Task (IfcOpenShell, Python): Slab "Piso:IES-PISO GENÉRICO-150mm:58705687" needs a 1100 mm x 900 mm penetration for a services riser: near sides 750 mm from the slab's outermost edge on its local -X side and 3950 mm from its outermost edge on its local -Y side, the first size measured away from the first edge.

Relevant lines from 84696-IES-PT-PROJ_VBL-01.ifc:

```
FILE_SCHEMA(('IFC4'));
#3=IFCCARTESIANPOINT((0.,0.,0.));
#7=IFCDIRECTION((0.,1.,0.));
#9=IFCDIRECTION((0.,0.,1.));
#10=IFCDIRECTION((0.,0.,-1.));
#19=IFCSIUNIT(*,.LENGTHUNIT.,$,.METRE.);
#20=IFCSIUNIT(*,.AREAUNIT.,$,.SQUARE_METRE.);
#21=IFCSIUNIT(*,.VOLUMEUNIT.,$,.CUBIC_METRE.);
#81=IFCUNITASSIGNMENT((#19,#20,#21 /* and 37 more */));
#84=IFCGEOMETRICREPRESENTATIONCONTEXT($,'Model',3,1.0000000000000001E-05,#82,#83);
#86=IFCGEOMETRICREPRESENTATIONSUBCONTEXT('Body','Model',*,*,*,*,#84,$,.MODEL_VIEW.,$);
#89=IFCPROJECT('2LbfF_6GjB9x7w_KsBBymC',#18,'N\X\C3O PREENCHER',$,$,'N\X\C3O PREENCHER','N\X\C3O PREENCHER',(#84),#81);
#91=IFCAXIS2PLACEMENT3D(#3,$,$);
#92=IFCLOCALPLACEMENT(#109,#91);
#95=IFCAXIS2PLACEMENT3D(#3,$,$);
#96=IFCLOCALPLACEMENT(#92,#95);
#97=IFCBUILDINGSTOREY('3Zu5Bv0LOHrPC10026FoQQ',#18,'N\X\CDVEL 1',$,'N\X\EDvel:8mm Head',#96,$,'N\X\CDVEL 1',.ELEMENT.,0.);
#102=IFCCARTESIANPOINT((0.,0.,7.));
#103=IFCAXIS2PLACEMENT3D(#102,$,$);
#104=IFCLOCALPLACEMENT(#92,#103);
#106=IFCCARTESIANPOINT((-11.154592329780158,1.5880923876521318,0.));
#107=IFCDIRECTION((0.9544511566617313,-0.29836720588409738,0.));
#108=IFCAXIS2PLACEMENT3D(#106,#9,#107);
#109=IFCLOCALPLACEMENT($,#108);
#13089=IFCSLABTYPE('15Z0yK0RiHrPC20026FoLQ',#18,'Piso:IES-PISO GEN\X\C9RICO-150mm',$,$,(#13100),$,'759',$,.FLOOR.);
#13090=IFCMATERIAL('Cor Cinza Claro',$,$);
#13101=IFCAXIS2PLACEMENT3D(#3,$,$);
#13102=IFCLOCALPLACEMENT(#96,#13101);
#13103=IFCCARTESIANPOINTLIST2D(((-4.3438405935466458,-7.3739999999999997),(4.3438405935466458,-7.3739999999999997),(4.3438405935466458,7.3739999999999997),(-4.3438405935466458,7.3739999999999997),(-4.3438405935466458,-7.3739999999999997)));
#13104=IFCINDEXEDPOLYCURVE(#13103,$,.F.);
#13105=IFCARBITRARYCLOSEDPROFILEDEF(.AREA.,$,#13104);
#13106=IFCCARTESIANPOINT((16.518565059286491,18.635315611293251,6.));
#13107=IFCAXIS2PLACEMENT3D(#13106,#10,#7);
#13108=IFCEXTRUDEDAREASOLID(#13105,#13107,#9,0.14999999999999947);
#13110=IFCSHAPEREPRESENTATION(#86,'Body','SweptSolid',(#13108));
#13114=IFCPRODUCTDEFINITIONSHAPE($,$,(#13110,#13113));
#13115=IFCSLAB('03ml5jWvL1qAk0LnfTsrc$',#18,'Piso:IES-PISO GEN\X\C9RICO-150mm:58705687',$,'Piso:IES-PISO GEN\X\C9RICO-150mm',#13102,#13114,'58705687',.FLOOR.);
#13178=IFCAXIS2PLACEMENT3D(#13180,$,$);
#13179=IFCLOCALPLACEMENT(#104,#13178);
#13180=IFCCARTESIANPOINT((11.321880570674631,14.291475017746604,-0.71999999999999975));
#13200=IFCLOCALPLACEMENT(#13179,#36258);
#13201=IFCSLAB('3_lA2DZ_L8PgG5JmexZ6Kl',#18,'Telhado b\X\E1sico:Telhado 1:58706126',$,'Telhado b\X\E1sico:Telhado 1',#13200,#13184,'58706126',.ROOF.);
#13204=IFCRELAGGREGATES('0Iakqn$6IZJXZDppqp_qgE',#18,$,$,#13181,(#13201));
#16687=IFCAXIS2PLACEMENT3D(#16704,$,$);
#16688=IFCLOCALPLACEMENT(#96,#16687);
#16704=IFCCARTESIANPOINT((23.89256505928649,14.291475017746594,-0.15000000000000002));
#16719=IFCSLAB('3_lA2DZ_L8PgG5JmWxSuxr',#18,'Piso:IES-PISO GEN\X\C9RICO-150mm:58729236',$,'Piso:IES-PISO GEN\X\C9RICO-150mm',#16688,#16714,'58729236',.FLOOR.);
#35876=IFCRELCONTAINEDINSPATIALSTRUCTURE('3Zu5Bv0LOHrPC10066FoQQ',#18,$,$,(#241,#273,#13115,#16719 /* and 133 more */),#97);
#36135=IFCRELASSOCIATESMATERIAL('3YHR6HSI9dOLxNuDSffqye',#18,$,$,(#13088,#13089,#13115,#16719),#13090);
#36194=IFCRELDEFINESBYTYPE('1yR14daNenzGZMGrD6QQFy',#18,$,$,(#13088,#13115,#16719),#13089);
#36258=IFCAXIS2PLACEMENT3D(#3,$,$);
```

```python
import numpy as np
import ifcopenshell
import ifcopenshell.api.feature
import ifcopenshell.api.geometry
import ifcopenshell.api.root
import ifcopenshell.geom
import ifcopenshell.util.placement
import ifcopenshell.util.representation
import ifcopenshell.util.shape
import ifcopenshell.util.unit

model = ifcopenshell.open("84696-IES-PT-PROJ_VBL-01.ifc")
unit_scale = ifcopenshell.util.unit.calculate_unit_scale(model)
settings = ifcopenshell.geom.settings()


def volume(element):
    """Net volume in cubic metres, openings subtracted."""
    shape = ifcopenshell.geom.create_shape(settings, element)
    return ifcopenshell.util.shape.get_volume(shape.geometry)


slab = model.by_guid("03ml5jWvL1qAk0LnfTsrc$")
before = volume(slab)

# Extent in the slab's own axes, in metres. The edges named are its -X and -Y sides.
slab_shape = ifcopenshell.geom.create_shape(settings, slab)
vertices = ifcopenshell.util.shape.get_vertices(slab_shape.geometry)
x_min, y_min, bottom = vertices.min(axis=0)
top = vertices[:, 2].max()

opening = ifcopenshell.api.root.create_entity(model, ifc_class="IfcOpeningElement", name="Services riser opening", predefined_type="OPENING")
context = ifcopenshell.util.representation.get_context(model, "Model", "Body", "MODEL_VIEW")
width, depth = 1.1, 0.9
outline = [(0.0, 0.0), (width, 0.0), (width, depth), (0.0, depth), (0.0, 0.0)]
# Overshoot both faces by 50 mm so the cut is clean.
shape = ifcopenshell.api.geometry.add_slab_representation(
    model, context=context, depth=top - bottom + 0.1, polyline=outline
)
ifcopenshell.api.geometry.assign_representation(model, product=opening, representation=shape)

matrix = ifcopenshell.util.placement.get_local_placement(slab.ObjectPlacement)
matrix[:, 3] = matrix @ np.append(np.array([x_min + 0.75, y_min + 3.95, bottom - 0.05]) / unit_scale, 1.0)
ifcopenshell.api.geometry.edit_object_placement(model, product=opening, matrix=matrix, is_si=False)
ifcopenshell.api.feature.add_feature(model, feature=opening, element=slab)

after = volume(slab)

print(f"slab volume {before:.3f} -> {after:.3f} m3")

model.write("84696-IES-PT-PROJ_VBL-01_updated.ifc")
```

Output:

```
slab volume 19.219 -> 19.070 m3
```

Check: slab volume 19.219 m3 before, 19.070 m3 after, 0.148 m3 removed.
